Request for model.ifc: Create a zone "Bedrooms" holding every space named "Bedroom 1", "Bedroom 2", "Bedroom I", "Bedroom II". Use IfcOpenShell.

First a look at what the model holds.

```python
import ifcopenshell

model = ifcopenshell.open("model.ifc")
print(model.schema)
seen = {}
for space in model.by_type("IfcSpace"):
    seen[space.LongName] = seen.get(space.LongName, 0) + 1
for name, count in sorted(seen.items(), key=str):
    print(count, "x", name)
print("zones:", [z.Name for z in model.by_type("IfcZone")][:20])
```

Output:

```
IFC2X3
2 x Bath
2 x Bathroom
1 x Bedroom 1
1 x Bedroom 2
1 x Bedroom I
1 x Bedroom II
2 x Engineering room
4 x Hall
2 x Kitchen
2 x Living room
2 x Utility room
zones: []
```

```python
import ifcopenshell
import ifcopenshell.api.group
import ifcopenshell.api.root

model = ifcopenshell.open("model.ifc")

names = {"Bedroom 1", "Bedroom 2", "Bedroom I", "Bedroom II"}
spaces = [s for s in model.by_type("IfcSpace") if s.LongName in names]

zone = ifcopenshell.api.root.create_entity(model, ifc_class="IfcZone", name="Bedrooms")
ifcopenshell.api.group.assign_group(model, products=spaces, group=zone)
print(len(spaces), "spaces in", zone.Name)

model.write("model_edited.ifc")
```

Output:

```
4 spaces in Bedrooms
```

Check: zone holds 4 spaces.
